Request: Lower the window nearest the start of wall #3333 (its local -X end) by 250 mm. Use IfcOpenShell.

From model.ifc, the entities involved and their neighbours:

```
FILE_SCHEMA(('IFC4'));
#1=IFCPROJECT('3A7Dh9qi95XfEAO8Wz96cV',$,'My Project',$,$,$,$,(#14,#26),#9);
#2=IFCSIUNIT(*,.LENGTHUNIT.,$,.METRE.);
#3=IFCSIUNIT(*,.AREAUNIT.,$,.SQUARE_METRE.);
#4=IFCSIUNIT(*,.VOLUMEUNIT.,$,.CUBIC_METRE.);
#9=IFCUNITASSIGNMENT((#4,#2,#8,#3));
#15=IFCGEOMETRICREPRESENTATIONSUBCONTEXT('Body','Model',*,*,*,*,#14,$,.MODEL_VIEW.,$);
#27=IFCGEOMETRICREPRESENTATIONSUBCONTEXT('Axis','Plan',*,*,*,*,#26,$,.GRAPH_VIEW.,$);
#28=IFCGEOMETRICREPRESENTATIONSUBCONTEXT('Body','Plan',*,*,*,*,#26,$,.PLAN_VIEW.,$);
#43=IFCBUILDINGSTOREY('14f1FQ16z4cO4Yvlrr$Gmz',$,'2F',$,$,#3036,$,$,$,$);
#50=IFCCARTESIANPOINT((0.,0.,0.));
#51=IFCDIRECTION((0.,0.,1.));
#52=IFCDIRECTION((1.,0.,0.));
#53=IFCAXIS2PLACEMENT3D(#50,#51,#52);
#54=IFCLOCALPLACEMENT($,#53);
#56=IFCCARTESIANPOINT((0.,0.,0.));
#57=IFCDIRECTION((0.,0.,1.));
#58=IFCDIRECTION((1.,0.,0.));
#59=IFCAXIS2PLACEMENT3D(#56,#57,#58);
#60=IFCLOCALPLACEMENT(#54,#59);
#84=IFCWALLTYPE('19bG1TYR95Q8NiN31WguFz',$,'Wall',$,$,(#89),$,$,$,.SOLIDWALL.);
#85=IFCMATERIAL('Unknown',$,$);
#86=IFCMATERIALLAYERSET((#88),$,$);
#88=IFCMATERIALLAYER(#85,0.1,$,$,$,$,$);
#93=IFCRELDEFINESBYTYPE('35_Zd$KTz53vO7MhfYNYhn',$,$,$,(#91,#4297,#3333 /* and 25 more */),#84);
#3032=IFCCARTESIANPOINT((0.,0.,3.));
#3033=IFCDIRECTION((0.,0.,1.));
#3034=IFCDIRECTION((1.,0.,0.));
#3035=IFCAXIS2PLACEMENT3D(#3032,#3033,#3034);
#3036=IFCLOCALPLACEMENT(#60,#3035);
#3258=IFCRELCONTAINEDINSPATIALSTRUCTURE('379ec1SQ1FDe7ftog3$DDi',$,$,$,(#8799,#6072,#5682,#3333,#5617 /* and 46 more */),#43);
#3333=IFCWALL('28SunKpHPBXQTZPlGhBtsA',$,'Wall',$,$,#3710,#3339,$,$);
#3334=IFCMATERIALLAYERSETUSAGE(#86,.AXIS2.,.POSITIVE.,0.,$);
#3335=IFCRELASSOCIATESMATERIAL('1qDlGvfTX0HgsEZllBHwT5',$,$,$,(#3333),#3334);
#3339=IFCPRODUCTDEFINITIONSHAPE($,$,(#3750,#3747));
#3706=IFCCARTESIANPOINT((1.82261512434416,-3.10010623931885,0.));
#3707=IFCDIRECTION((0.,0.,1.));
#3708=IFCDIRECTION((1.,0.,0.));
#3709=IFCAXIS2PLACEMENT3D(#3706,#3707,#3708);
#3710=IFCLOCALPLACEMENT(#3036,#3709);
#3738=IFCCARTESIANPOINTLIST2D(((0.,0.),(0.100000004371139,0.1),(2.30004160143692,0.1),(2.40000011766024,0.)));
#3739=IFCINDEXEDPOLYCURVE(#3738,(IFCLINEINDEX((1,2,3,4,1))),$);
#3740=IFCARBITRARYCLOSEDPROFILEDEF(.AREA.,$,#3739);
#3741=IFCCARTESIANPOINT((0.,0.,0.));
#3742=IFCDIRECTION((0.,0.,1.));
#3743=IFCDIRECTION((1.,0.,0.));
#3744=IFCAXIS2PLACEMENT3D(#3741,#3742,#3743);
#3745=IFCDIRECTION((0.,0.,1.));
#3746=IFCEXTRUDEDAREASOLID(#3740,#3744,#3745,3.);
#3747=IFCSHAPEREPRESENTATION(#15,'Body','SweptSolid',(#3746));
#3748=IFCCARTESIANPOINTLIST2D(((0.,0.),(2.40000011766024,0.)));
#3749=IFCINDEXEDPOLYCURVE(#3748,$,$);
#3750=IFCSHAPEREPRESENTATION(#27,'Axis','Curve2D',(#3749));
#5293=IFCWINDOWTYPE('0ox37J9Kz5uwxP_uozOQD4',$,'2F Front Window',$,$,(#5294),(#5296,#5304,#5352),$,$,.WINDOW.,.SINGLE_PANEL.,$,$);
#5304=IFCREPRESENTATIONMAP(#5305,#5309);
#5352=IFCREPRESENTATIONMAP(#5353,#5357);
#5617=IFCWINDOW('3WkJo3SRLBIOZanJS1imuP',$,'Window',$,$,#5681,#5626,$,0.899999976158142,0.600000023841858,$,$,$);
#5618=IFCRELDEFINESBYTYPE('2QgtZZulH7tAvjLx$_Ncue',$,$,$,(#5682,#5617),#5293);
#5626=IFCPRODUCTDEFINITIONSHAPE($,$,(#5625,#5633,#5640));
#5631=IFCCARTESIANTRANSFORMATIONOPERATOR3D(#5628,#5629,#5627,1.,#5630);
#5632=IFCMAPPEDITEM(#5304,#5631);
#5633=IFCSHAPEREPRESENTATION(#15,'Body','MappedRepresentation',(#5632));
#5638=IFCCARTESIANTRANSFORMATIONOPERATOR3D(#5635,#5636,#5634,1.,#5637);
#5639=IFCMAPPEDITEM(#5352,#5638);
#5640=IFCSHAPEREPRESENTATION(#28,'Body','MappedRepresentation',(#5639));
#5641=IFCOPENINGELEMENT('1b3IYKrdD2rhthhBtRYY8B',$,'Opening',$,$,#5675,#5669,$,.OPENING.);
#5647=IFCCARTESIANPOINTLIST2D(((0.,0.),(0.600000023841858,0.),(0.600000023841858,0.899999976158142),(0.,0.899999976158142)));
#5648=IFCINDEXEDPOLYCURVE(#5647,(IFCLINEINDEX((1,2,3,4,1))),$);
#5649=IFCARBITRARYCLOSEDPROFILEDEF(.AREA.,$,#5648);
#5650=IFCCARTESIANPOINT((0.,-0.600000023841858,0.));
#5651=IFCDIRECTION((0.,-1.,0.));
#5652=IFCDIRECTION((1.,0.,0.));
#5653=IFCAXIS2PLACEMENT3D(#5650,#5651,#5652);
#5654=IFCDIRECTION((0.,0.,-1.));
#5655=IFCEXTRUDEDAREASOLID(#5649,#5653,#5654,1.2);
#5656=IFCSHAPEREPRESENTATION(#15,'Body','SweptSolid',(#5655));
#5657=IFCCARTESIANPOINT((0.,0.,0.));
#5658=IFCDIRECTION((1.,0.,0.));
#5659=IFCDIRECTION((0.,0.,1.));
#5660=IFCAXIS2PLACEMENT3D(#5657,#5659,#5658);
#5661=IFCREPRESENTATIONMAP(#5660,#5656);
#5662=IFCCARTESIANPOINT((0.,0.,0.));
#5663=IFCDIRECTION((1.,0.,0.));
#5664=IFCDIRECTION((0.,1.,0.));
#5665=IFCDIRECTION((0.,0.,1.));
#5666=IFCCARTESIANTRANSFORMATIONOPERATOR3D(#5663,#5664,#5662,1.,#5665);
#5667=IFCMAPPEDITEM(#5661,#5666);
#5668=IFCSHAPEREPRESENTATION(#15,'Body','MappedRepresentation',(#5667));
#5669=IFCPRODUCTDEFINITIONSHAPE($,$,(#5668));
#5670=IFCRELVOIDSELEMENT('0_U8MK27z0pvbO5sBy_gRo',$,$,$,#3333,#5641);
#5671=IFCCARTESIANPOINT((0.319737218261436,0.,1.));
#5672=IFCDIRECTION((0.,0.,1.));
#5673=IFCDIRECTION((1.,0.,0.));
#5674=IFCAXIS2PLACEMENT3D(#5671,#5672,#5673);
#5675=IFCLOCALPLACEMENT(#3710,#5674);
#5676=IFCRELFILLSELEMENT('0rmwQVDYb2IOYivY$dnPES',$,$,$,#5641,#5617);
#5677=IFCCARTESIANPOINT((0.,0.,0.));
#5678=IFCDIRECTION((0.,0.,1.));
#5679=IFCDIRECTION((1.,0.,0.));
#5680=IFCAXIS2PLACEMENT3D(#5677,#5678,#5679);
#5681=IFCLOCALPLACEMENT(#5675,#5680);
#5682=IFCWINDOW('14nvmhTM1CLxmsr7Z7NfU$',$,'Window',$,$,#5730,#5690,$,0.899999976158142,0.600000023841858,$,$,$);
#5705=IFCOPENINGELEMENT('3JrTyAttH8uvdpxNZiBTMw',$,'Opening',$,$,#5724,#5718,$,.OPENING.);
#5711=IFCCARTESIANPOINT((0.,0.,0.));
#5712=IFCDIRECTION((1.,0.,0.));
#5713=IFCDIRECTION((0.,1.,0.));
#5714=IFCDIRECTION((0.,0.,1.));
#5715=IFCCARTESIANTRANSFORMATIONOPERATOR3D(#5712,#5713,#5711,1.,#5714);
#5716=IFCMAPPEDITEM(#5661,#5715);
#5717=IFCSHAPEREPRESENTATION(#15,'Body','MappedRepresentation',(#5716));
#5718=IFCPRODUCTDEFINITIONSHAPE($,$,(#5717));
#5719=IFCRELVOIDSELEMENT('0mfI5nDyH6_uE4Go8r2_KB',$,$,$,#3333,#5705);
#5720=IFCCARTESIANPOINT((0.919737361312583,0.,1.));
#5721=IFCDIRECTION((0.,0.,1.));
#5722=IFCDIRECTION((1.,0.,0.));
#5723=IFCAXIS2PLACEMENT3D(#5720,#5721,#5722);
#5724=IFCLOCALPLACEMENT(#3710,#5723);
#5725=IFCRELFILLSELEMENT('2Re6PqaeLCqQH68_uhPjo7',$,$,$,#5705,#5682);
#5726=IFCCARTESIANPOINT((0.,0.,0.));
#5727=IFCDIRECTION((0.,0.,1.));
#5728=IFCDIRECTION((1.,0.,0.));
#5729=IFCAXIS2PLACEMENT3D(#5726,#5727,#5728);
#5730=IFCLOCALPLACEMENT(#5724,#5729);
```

```python
import numpy as np
import ifcopenshell
import ifcopenshell.api.geometry
import ifcopenshell.util.placement
import ifcopenshell.util.unit

model = ifcopenshell.open("model.ifc")
unit_scale = ifcopenshell.util.unit.calculate_unit_scale(model)

window = model.by_guid("3WkJo3SRLBIOZanJS1imuP")
opening = window.FillsVoids[0].RelatingOpeningElement
dz = -0.25 / unit_scale

shift = np.array([0.0, 0.0, dz])
# The window is placed relative to its opening, so it follows when the opening moves.
matrix = ifcopenshell.util.placement.get_local_placement(opening.ObjectPlacement)
matrix[:3, 3] += shift
ifcopenshell.api.geometry.edit_object_placement(
    model, product=opening, matrix=matrix, is_si=False, should_transform_children=True
)

print(f"moved by {dz * unit_scale:+.3f} m")

model.write("model-out.ifc")
```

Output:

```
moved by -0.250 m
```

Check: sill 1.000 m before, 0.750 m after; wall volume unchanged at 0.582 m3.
